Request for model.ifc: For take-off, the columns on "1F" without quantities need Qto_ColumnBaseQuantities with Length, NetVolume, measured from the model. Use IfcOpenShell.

First a look at what the model holds.

```python
import ifcopenshell
import ifcopenshell.util.element
import ifcopenshell.util.unit

model = ifcopenshell.open("model.ifc")
print(model.schema)
for unit_type in ("LENGTHUNIT", "AREAUNIT", "VOLUMEUNIT"):
    print(unit_type, ifcopenshell.util.unit.calculate_unit_scale(model, unit_type))
storey = next(s for s in model.by_type("IfcBuildingStorey") if s.Name == "1F")
columns = [e for e in ifcopenshell.util.element.get_decomposition(storey) if e.is_a("IfcColumn")]
for e in sorted(columns, key=lambda e: e.id()):
    print(e.id(), e.is_a(), e.Name, list(ifcopenshell.util.element.get_psets(e, qtos_only=True)), sep=" | ")
```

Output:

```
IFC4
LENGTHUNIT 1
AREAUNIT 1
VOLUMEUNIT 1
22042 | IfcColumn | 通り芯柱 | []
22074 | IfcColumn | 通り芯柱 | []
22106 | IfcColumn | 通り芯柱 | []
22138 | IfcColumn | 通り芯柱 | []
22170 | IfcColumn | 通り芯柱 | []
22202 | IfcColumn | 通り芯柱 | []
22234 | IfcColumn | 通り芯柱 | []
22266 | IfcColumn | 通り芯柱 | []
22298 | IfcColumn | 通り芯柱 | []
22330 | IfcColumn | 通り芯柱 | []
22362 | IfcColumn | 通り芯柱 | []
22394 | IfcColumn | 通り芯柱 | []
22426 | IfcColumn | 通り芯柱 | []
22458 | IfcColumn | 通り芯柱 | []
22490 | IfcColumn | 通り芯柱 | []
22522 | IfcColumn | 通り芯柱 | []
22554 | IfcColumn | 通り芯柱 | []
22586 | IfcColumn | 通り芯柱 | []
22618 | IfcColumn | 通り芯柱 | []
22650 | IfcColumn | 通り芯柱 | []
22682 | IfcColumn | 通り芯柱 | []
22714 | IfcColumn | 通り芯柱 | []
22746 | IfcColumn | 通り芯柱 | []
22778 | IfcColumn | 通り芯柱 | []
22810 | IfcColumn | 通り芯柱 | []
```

```python
import ifcopenshell
import ifcopenshell.api.pset
import ifcopenshell.geom
import ifcopenshell.util.element
import ifcopenshell.util.shape
import ifcopenshell.util.unit

model = ifcopenshell.open("model.ifc")
unit_scale = ifcopenshell.util.unit.calculate_unit_scale(model)
volume_scale = ifcopenshell.util.unit.calculate_unit_scale(model, "VOLUMEUNIT")
settings = ifcopenshell.geom.settings()

storey = next(s for s in model.by_type("IfcBuildingStorey") if s.Name == "1F")
columns = [e for e in ifcopenshell.util.element.get_decomposition(storey) if e.is_a("IfcColumn")]

for e in sorted(columns, key=lambda e: e.id()):
    if ifcopenshell.util.element.get_psets(e, qtos_only=True, should_inherit=False):
        continue
    # Geometry comes back in metres, in the element's own axes.
    shape = ifcopenshell.geom.create_shape(settings, e)
    values = {
        "Length": ifcopenshell.util.shape.get_z(shape.geometry) / unit_scale,
        "NetVolume": ifcopenshell.util.shape.get_volume(shape.geometry) / volume_scale,
    }
    qto = ifcopenshell.api.pset.add_qto(model, product=e, name="Qto_ColumnBaseQuantities")
    ifcopenshell.api.pset.edit_qto(model, qto=qto, properties=values)
    print(e.id(), {k: round(v, 3) for k, v in values.items()})

model.write("model_updated.ifc")
```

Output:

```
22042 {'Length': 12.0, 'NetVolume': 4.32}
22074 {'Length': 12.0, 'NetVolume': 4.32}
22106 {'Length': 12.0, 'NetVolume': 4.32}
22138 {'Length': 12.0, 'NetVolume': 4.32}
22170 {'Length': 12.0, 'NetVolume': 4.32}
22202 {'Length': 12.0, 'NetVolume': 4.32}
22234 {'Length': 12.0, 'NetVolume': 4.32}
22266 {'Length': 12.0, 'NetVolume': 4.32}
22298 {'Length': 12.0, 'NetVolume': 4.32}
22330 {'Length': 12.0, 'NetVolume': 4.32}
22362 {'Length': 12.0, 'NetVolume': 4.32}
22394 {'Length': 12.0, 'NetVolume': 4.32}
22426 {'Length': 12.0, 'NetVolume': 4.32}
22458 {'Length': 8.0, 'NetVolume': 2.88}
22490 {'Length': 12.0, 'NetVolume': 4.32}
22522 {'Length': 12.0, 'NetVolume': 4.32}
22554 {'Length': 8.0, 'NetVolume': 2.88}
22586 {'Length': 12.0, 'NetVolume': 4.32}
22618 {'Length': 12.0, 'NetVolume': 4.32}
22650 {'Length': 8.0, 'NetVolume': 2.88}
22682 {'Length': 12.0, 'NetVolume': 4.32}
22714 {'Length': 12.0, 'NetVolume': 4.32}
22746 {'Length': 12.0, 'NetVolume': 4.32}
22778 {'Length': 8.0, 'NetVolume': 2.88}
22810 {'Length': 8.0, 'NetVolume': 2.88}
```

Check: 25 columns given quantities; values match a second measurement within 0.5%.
